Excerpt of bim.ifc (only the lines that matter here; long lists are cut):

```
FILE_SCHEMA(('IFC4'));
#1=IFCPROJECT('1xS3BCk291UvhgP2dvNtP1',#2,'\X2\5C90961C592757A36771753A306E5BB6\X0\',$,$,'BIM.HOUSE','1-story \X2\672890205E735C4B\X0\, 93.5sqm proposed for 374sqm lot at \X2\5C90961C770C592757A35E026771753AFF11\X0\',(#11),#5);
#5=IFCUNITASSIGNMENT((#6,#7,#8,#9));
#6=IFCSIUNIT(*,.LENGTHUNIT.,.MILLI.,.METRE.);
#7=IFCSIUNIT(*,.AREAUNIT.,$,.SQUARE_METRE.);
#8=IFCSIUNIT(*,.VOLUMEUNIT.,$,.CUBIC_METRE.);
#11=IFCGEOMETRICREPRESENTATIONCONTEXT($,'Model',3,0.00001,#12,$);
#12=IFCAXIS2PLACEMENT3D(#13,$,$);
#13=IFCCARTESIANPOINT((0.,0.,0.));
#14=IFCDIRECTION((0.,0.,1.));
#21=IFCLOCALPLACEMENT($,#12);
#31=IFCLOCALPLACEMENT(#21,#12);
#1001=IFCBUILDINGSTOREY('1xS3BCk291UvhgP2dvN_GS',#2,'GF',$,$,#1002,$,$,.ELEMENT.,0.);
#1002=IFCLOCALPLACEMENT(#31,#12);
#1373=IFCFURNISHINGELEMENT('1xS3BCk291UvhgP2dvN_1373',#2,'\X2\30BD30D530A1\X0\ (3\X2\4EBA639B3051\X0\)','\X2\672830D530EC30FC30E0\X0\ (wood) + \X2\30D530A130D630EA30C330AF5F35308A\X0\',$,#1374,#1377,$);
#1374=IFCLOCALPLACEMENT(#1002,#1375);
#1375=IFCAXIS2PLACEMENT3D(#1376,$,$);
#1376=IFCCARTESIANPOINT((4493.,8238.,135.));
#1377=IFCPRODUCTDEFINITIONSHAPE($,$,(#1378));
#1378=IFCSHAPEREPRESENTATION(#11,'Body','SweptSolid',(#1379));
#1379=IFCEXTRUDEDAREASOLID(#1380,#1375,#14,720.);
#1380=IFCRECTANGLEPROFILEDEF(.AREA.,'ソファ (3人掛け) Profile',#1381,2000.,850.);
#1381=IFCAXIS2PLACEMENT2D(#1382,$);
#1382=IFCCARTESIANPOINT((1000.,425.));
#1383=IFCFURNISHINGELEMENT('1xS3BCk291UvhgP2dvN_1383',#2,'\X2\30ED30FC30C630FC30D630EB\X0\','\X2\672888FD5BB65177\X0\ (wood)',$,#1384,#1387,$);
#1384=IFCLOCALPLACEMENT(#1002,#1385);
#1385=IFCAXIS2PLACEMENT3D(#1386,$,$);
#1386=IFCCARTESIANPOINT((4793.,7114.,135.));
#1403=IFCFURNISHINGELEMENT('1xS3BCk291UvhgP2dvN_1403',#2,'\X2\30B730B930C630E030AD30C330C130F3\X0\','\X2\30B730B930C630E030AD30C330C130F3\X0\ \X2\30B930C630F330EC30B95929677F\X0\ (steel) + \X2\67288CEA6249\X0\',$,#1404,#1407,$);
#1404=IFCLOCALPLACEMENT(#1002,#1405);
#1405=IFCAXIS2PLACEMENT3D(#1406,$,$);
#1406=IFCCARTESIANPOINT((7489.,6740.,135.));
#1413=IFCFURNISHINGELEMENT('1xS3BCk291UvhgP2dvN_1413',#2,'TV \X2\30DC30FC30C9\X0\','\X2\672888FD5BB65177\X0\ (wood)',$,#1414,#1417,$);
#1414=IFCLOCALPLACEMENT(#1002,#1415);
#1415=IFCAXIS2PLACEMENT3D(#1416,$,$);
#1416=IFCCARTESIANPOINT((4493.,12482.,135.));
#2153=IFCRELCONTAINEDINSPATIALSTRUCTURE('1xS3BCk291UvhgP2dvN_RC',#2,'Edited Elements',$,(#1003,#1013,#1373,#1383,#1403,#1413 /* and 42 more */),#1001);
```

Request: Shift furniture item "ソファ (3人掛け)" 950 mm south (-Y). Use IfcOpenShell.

```python
import ifcopenshell
import ifcopenshell.api.geometry
import ifcopenshell.util.placement

model = ifcopenshell.open("bim.ifc")

item = model.by_guid("1xS3BCk291UvhgP2dvN_1373")
matrix = ifcopenshell.util.placement.get_local_placement(item.ObjectPlacement)
matrix[1, 3] -= 950.0
ifcopenshell.api.geometry.edit_object_placement(model, product=item, matrix=matrix, is_si=False)

print(ifcopenshell.util.placement.get_local_placement(item.ObjectPlacement).round(3) + 0.0)

model.write("bim-out.ifc")
```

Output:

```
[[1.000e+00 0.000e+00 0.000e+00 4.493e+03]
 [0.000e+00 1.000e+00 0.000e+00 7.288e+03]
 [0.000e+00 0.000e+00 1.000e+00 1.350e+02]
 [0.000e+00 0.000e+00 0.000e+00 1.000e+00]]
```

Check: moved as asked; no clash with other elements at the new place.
